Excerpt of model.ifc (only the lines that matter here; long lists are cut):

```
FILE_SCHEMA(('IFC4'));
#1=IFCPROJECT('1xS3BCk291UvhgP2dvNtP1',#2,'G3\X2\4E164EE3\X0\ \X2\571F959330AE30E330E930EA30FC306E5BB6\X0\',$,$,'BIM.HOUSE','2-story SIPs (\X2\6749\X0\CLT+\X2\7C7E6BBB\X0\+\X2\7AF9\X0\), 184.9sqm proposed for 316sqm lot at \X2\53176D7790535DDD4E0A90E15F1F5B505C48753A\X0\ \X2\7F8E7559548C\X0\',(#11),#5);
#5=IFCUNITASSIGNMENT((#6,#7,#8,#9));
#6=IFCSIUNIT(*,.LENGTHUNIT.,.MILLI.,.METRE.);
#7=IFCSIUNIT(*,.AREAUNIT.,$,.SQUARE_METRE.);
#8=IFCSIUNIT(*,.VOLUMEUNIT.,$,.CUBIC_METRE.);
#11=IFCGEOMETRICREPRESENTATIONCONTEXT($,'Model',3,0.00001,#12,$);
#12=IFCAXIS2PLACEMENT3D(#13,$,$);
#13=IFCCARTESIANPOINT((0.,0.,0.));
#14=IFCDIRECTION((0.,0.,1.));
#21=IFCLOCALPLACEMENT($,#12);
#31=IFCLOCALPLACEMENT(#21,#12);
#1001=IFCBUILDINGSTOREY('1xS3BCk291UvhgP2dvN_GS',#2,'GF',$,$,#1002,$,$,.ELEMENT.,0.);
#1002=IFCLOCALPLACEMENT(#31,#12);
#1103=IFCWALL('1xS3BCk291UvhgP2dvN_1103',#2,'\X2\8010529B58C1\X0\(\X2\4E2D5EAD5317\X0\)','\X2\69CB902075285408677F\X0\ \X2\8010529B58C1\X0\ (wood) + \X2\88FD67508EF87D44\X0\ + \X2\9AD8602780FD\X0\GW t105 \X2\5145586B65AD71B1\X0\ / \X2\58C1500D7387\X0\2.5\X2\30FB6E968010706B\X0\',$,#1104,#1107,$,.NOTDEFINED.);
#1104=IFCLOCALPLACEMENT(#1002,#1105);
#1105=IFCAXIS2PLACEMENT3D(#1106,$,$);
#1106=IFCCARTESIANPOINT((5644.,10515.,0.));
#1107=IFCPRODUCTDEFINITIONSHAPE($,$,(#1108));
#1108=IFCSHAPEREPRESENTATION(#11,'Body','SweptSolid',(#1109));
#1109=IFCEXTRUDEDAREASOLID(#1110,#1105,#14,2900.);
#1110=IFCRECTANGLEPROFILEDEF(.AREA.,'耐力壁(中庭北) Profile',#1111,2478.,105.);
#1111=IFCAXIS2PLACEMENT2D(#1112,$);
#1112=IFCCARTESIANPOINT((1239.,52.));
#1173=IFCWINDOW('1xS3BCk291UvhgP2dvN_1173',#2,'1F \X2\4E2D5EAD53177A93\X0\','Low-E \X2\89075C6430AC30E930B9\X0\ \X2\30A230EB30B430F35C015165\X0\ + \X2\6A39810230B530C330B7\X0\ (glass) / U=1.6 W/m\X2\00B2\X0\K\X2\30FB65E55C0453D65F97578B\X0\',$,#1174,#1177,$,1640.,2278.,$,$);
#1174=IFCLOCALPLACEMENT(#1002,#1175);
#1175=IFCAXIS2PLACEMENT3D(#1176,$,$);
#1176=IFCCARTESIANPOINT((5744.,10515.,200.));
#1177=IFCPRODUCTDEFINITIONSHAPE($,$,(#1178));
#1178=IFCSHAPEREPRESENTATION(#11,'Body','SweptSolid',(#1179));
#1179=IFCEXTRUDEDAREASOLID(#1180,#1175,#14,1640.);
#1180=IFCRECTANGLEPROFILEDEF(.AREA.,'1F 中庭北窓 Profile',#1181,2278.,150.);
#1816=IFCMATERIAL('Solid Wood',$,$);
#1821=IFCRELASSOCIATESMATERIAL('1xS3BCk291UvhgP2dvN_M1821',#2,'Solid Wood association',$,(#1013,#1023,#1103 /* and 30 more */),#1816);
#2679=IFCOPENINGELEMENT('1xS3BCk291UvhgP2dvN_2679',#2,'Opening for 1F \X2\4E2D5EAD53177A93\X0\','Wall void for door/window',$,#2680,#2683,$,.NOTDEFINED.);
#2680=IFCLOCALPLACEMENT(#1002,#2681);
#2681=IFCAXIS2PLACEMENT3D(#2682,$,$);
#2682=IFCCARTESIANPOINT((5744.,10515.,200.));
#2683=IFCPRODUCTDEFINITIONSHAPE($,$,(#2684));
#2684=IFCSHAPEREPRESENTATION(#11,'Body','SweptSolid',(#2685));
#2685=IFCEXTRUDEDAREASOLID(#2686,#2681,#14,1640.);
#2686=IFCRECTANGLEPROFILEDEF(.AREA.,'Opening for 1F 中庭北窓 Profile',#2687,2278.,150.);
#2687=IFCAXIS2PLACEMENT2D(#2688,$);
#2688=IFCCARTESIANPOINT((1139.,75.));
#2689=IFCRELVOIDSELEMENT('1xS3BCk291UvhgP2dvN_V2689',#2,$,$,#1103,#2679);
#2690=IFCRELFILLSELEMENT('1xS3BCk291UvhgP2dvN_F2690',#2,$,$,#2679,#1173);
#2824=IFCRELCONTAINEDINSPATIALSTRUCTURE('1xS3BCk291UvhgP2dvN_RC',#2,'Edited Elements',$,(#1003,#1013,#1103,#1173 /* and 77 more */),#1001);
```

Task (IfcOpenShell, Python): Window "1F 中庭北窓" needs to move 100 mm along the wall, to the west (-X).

```python
import ifcopenshell
import ifcopenshell.api.geometry
import ifcopenshell.util.placement
import ifcopenshell.util.unit

model = ifcopenshell.open("model.ifc")
unit_scale = ifcopenshell.util.unit.calculate_unit_scale(model)

window = model.by_id(1173)
opening = window.FillsVoids[0].RelatingOpeningElement
wall = opening.VoidsElements[0].RelatingBuildingElement

wall_matrix = ifcopenshell.util.placement.get_local_placement(wall.ObjectPlacement)
shift = wall_matrix[:3, 0] * -0.1 / unit_scale
before = ifcopenshell.util.placement.get_local_placement(window.ObjectPlacement)[:3, 3].copy()

# The window is not placed relative to its opening, so move both.
for product in (opening, window):
    matrix = ifcopenshell.util.placement.get_local_placement(product.ObjectPlacement)
    matrix[:3, 3] += shift
    ifcopenshell.api.geometry.edit_object_placement(model, product=product, matrix=matrix, is_si=False)

after = ifcopenshell.util.placement.get_local_placement(window.ObjectPlacement)[:3, 3]
print("window moved by", (after - before).round(3) + 0.0)

model.write("model_edited.ifc")
```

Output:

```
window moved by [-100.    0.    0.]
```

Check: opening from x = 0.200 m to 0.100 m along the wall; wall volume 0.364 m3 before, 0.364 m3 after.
